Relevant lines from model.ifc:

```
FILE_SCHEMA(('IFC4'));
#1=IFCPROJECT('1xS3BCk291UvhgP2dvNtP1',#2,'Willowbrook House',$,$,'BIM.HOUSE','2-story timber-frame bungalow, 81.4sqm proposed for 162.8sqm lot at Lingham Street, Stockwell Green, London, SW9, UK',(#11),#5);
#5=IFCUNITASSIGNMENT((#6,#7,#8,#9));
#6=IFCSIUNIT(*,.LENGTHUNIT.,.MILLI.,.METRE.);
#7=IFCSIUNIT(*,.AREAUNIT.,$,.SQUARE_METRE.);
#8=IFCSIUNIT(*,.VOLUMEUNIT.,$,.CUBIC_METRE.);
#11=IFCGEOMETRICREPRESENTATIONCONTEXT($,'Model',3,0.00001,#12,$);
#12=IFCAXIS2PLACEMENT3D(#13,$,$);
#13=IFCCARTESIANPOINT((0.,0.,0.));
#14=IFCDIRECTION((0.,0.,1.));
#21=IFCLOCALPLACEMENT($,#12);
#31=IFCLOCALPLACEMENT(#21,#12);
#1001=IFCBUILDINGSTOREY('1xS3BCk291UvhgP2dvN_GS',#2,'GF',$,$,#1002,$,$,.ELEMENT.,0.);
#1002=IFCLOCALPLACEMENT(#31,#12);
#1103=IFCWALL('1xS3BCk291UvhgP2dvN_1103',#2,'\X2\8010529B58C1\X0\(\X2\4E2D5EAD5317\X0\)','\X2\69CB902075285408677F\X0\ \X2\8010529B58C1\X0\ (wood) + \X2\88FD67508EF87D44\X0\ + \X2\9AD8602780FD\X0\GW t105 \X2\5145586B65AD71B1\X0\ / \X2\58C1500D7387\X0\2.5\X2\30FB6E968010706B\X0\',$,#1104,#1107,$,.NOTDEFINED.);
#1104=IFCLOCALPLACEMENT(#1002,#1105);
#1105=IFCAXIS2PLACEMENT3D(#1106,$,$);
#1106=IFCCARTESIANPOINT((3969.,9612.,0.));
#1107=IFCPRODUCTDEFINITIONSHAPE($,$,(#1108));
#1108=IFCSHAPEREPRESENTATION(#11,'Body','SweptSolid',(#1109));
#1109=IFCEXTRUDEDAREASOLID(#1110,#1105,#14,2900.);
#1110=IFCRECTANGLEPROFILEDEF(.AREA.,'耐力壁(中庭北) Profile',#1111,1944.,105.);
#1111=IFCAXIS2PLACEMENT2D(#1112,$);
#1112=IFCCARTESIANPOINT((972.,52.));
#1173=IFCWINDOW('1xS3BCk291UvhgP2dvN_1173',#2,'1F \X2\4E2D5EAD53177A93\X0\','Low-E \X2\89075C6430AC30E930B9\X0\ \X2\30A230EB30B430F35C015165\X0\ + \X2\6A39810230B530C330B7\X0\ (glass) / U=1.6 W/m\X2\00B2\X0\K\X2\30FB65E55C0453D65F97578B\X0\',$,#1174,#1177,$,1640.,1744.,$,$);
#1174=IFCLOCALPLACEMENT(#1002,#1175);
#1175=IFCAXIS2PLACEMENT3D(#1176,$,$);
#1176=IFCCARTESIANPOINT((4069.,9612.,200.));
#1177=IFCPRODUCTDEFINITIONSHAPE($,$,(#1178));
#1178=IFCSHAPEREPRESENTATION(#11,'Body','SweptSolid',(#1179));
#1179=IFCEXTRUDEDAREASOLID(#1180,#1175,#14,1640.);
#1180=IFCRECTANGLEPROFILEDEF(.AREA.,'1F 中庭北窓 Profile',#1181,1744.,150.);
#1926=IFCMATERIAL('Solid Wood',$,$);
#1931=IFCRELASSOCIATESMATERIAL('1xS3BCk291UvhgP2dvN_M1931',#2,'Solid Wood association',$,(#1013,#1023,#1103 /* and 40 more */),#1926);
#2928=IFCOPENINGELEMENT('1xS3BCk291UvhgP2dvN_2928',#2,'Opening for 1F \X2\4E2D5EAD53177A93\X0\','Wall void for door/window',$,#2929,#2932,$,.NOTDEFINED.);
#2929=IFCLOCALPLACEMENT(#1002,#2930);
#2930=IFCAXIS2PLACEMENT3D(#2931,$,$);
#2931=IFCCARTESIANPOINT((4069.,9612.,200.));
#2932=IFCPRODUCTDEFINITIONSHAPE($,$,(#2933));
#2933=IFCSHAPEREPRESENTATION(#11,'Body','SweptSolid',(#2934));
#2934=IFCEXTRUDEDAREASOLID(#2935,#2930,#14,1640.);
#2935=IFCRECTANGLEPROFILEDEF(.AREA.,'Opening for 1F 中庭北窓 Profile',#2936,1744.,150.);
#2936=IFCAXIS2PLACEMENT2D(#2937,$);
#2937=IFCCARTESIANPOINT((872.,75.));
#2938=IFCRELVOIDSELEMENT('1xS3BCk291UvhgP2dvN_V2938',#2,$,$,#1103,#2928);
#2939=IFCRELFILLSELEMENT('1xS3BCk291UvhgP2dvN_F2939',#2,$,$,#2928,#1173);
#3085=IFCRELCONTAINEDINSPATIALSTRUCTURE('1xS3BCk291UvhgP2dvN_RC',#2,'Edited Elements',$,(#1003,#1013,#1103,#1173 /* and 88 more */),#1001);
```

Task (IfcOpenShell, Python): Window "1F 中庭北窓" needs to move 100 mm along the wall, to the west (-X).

```python
import ifcopenshell
import ifcopenshell.api.geometry
import ifcopenshell.util.placement
import ifcopenshell.util.unit

model = ifcopenshell.open("model.ifc")
unit_scale = ifcopenshell.util.unit.calculate_unit_scale(model)

window = model.by_id(1173)
opening = window.FillsVoids[0].RelatingOpeningElement
wall = opening.VoidsElements[0].RelatingBuildingElement

wall_matrix = ifcopenshell.util.placement.get_local_placement(wall.ObjectPlacement)
shift = wall_matrix[:3, 0] * -0.1 / unit_scale
before = ifcopenshell.util.placement.get_local_placement(window.ObjectPlacement)[:3, 3].copy()

# The window is not placed relative to its opening, so move both.
for product in (opening, window):
    matrix = ifcopenshell.util.placement.get_local_placement(product.ObjectPlacement)
    matrix[:3, 3] += shift
    ifcopenshell.api.geometry.edit_object_placement(model, product=product, matrix=matrix, is_si=False)

after = ifcopenshell.util.placement.get_local_placement(window.ObjectPlacement)[:3, 3]
print("window moved by", (after - before).round(3) + 0.0)

model.write("model_edited.ifc")
```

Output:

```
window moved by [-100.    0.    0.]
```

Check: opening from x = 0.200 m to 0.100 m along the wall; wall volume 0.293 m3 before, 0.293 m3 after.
